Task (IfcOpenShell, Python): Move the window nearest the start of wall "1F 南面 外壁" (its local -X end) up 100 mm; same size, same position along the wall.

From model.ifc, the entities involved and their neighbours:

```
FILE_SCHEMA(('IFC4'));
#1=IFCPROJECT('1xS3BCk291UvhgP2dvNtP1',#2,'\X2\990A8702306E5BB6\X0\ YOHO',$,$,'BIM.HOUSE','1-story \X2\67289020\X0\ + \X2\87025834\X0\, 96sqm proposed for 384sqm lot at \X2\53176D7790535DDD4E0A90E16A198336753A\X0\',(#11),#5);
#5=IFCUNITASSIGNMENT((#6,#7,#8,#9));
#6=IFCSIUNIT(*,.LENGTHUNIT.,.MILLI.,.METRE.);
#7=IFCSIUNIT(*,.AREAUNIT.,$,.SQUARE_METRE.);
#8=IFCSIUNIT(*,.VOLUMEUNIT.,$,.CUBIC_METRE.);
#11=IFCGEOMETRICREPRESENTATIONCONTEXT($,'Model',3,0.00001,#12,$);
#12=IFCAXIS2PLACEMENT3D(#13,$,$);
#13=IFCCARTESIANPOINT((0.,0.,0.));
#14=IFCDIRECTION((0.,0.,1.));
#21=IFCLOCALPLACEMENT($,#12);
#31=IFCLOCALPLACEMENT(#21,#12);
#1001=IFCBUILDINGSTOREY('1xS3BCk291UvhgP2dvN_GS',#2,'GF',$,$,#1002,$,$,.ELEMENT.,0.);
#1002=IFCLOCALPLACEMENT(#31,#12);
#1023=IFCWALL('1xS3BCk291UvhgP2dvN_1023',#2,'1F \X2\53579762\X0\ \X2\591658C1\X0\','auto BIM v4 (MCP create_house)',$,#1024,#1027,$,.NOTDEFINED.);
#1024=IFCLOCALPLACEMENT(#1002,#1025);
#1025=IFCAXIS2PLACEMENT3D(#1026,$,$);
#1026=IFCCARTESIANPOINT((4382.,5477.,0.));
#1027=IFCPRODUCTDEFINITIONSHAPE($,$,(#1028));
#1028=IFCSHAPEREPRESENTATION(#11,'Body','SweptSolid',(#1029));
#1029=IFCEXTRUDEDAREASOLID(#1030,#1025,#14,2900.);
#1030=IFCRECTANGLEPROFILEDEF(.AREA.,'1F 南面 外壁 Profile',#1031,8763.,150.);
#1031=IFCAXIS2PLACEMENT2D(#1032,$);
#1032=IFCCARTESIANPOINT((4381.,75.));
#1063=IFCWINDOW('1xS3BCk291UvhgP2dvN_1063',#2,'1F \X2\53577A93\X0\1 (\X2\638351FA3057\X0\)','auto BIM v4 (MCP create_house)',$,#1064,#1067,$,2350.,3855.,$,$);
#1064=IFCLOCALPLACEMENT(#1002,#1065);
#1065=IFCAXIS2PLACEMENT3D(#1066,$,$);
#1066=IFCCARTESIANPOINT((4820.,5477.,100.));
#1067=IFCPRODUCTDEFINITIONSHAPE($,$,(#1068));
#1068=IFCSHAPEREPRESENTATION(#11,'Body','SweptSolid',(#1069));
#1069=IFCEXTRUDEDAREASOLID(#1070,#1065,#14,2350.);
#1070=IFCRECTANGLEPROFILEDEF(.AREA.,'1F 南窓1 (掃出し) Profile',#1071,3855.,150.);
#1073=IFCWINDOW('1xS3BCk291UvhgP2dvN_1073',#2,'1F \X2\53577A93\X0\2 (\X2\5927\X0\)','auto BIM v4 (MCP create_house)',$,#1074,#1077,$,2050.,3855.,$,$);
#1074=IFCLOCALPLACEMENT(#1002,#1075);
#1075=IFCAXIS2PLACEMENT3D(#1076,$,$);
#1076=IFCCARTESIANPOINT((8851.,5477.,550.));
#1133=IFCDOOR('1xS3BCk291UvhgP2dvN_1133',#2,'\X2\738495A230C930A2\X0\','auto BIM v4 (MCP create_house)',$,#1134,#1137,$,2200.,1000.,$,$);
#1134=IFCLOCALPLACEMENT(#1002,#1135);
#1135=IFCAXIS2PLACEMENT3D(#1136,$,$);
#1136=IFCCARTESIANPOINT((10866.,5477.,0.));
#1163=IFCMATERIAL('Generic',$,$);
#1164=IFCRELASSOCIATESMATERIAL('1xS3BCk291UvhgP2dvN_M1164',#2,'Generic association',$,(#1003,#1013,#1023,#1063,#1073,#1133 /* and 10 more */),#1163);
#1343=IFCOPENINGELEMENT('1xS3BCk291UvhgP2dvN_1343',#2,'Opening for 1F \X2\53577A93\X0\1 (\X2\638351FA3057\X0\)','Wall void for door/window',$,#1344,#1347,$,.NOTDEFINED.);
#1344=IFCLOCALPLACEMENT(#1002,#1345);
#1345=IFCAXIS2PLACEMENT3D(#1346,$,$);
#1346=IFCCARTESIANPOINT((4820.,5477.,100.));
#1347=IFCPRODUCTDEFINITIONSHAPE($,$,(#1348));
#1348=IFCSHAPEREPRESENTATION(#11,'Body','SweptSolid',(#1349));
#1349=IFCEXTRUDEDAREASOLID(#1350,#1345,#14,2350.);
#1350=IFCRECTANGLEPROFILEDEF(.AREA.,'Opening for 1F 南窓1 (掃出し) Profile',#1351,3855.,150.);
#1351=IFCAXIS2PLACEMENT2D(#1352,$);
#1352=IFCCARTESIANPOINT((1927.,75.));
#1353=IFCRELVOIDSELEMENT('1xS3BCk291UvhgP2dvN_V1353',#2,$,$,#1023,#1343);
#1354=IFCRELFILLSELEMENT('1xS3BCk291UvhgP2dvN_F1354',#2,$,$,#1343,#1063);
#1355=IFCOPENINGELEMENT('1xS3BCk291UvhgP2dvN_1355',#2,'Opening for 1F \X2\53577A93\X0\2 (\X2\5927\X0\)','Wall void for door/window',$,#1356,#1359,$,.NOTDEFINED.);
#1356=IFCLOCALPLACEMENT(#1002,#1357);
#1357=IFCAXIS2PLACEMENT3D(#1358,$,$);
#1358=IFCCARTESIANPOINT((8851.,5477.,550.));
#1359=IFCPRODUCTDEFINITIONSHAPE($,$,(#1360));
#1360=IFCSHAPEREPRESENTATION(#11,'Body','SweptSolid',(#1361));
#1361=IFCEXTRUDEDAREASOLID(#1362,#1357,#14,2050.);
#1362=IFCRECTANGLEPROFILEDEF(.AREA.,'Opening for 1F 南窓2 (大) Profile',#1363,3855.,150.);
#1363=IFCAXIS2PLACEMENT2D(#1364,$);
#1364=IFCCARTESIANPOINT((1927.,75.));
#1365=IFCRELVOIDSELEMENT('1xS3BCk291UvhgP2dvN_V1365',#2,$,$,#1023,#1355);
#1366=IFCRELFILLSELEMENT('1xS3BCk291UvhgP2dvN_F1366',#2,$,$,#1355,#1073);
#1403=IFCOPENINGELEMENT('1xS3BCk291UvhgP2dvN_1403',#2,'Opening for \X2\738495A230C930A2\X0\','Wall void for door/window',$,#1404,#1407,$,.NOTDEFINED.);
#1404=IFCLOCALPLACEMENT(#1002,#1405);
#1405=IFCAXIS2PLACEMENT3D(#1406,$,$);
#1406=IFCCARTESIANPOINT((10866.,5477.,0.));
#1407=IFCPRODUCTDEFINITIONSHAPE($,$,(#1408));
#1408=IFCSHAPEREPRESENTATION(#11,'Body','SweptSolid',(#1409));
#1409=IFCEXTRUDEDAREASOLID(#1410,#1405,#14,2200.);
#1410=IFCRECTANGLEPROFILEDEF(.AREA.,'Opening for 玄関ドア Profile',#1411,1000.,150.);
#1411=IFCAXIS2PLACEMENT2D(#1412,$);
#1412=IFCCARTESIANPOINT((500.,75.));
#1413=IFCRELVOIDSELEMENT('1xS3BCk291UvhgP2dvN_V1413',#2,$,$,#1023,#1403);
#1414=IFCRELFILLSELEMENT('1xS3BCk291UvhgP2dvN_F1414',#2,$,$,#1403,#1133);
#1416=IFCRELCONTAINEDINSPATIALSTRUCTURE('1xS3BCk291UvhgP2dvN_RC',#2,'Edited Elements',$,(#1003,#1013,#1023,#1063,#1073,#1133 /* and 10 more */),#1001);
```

```python
import numpy as np
import ifcopenshell
import ifcopenshell.api.geometry
import ifcopenshell.util.placement
import ifcopenshell.util.unit

model = ifcopenshell.open("model.ifc")
unit_scale = ifcopenshell.util.unit.calculate_unit_scale(model)

window = model.by_guid("1xS3BCk291UvhgP2dvN_1063")
opening = window.FillsVoids[0].RelatingOpeningElement
dz = 0.1 / unit_scale

shift = np.array([0.0, 0.0, dz])
# The window is not placed relative to its opening, so move both.
for product in (opening, window):
    matrix = ifcopenshell.util.placement.get_local_placement(product.ObjectPlacement)
    matrix[:3, 3] += shift
    ifcopenshell.api.geometry.edit_object_placement(model, product=product, matrix=matrix, is_si=False)

print(f"moved by {dz * unit_scale:+.3f} m")

model.write("model-out.ifc")
```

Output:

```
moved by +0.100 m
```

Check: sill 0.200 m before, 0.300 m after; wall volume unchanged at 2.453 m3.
